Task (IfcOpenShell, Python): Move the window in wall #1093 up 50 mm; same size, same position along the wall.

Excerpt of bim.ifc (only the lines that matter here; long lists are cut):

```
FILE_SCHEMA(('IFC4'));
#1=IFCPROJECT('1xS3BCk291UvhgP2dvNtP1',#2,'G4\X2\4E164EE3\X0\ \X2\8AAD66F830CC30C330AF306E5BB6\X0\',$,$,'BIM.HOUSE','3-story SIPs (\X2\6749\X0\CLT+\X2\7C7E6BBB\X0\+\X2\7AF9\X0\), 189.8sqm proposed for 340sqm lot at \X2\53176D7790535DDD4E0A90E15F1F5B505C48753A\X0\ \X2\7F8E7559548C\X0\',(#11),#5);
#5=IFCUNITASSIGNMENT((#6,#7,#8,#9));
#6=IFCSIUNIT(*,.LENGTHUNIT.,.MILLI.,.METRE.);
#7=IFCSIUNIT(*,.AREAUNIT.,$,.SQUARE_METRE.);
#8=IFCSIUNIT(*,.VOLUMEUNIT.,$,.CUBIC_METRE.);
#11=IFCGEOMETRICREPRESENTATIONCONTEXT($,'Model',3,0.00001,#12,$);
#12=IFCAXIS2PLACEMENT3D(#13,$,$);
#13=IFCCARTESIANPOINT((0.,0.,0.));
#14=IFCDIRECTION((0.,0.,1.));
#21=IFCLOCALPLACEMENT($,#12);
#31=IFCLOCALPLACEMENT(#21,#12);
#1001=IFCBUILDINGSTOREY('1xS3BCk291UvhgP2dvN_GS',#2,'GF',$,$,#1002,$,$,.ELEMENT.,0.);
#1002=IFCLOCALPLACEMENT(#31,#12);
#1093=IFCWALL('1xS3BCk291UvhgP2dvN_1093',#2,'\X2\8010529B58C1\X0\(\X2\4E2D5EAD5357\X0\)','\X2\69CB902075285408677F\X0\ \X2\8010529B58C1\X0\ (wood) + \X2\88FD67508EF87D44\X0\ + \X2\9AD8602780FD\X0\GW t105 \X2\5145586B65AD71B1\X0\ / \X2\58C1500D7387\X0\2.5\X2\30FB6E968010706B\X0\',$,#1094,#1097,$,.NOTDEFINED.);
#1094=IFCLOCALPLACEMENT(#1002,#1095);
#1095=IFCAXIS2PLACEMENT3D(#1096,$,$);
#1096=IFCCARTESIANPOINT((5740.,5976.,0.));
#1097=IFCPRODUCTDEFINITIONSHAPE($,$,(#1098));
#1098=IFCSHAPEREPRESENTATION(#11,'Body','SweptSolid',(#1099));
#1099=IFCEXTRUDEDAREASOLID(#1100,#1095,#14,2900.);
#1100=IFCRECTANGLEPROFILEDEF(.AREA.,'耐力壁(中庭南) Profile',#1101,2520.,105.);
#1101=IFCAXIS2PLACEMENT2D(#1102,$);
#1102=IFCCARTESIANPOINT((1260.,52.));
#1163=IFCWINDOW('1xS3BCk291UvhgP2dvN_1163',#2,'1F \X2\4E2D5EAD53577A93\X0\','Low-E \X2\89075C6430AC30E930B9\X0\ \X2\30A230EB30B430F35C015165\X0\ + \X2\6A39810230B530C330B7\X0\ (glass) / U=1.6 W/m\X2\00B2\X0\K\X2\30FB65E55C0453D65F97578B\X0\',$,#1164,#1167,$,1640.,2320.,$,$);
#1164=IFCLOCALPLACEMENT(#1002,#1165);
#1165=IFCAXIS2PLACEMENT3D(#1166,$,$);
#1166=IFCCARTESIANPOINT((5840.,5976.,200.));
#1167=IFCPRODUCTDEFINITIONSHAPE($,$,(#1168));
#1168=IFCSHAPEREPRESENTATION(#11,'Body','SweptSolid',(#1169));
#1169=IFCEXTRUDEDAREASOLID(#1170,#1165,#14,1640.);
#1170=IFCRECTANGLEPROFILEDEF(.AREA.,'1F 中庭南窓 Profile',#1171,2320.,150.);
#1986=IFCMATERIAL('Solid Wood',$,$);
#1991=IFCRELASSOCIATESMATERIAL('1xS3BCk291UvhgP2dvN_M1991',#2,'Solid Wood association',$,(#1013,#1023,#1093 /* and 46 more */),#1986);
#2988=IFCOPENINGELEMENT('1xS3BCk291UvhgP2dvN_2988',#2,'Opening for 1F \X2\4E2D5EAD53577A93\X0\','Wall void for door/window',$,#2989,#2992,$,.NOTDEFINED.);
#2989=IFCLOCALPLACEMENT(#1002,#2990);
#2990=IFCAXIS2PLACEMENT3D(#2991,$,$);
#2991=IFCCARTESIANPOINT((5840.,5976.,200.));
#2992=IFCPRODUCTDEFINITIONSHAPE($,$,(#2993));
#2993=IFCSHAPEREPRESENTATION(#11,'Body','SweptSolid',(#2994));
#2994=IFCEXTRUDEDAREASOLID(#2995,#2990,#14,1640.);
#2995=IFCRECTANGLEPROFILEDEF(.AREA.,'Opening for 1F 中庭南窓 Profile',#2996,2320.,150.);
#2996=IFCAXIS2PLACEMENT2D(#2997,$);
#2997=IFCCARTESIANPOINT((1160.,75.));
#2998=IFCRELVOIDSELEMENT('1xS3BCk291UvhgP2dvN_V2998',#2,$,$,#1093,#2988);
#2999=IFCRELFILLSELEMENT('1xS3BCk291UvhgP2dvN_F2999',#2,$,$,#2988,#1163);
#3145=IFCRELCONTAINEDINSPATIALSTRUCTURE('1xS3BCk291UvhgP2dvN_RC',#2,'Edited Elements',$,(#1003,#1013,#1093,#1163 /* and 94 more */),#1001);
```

```python
import numpy as np
import ifcopenshell
import ifcopenshell.api.geometry
import ifcopenshell.util.placement
import ifcopenshell.util.unit

model = ifcopenshell.open("bim.ifc")
unit_scale = ifcopenshell.util.unit.calculate_unit_scale(model)

window = model.by_guid("1xS3BCk291UvhgP2dvN_1163")
opening = window.FillsVoids[0].RelatingOpeningElement
dz = 50.0

shift = np.array([0.0, 0.0, dz])
# The window is not placed relative to its opening, so move both.
for product in (opening, window):
    matrix = ifcopenshell.util.placement.get_local_placement(product.ObjectPlacement)
    matrix[:3, 3] += shift
    ifcopenshell.api.geometry.edit_object_placement(model, product=product, matrix=matrix, is_si=False)

print(f"moved by {dz * unit_scale:+.3f} m")

model.write("bim_updated.ifc")
```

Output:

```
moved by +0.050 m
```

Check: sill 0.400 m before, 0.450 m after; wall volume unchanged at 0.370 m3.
